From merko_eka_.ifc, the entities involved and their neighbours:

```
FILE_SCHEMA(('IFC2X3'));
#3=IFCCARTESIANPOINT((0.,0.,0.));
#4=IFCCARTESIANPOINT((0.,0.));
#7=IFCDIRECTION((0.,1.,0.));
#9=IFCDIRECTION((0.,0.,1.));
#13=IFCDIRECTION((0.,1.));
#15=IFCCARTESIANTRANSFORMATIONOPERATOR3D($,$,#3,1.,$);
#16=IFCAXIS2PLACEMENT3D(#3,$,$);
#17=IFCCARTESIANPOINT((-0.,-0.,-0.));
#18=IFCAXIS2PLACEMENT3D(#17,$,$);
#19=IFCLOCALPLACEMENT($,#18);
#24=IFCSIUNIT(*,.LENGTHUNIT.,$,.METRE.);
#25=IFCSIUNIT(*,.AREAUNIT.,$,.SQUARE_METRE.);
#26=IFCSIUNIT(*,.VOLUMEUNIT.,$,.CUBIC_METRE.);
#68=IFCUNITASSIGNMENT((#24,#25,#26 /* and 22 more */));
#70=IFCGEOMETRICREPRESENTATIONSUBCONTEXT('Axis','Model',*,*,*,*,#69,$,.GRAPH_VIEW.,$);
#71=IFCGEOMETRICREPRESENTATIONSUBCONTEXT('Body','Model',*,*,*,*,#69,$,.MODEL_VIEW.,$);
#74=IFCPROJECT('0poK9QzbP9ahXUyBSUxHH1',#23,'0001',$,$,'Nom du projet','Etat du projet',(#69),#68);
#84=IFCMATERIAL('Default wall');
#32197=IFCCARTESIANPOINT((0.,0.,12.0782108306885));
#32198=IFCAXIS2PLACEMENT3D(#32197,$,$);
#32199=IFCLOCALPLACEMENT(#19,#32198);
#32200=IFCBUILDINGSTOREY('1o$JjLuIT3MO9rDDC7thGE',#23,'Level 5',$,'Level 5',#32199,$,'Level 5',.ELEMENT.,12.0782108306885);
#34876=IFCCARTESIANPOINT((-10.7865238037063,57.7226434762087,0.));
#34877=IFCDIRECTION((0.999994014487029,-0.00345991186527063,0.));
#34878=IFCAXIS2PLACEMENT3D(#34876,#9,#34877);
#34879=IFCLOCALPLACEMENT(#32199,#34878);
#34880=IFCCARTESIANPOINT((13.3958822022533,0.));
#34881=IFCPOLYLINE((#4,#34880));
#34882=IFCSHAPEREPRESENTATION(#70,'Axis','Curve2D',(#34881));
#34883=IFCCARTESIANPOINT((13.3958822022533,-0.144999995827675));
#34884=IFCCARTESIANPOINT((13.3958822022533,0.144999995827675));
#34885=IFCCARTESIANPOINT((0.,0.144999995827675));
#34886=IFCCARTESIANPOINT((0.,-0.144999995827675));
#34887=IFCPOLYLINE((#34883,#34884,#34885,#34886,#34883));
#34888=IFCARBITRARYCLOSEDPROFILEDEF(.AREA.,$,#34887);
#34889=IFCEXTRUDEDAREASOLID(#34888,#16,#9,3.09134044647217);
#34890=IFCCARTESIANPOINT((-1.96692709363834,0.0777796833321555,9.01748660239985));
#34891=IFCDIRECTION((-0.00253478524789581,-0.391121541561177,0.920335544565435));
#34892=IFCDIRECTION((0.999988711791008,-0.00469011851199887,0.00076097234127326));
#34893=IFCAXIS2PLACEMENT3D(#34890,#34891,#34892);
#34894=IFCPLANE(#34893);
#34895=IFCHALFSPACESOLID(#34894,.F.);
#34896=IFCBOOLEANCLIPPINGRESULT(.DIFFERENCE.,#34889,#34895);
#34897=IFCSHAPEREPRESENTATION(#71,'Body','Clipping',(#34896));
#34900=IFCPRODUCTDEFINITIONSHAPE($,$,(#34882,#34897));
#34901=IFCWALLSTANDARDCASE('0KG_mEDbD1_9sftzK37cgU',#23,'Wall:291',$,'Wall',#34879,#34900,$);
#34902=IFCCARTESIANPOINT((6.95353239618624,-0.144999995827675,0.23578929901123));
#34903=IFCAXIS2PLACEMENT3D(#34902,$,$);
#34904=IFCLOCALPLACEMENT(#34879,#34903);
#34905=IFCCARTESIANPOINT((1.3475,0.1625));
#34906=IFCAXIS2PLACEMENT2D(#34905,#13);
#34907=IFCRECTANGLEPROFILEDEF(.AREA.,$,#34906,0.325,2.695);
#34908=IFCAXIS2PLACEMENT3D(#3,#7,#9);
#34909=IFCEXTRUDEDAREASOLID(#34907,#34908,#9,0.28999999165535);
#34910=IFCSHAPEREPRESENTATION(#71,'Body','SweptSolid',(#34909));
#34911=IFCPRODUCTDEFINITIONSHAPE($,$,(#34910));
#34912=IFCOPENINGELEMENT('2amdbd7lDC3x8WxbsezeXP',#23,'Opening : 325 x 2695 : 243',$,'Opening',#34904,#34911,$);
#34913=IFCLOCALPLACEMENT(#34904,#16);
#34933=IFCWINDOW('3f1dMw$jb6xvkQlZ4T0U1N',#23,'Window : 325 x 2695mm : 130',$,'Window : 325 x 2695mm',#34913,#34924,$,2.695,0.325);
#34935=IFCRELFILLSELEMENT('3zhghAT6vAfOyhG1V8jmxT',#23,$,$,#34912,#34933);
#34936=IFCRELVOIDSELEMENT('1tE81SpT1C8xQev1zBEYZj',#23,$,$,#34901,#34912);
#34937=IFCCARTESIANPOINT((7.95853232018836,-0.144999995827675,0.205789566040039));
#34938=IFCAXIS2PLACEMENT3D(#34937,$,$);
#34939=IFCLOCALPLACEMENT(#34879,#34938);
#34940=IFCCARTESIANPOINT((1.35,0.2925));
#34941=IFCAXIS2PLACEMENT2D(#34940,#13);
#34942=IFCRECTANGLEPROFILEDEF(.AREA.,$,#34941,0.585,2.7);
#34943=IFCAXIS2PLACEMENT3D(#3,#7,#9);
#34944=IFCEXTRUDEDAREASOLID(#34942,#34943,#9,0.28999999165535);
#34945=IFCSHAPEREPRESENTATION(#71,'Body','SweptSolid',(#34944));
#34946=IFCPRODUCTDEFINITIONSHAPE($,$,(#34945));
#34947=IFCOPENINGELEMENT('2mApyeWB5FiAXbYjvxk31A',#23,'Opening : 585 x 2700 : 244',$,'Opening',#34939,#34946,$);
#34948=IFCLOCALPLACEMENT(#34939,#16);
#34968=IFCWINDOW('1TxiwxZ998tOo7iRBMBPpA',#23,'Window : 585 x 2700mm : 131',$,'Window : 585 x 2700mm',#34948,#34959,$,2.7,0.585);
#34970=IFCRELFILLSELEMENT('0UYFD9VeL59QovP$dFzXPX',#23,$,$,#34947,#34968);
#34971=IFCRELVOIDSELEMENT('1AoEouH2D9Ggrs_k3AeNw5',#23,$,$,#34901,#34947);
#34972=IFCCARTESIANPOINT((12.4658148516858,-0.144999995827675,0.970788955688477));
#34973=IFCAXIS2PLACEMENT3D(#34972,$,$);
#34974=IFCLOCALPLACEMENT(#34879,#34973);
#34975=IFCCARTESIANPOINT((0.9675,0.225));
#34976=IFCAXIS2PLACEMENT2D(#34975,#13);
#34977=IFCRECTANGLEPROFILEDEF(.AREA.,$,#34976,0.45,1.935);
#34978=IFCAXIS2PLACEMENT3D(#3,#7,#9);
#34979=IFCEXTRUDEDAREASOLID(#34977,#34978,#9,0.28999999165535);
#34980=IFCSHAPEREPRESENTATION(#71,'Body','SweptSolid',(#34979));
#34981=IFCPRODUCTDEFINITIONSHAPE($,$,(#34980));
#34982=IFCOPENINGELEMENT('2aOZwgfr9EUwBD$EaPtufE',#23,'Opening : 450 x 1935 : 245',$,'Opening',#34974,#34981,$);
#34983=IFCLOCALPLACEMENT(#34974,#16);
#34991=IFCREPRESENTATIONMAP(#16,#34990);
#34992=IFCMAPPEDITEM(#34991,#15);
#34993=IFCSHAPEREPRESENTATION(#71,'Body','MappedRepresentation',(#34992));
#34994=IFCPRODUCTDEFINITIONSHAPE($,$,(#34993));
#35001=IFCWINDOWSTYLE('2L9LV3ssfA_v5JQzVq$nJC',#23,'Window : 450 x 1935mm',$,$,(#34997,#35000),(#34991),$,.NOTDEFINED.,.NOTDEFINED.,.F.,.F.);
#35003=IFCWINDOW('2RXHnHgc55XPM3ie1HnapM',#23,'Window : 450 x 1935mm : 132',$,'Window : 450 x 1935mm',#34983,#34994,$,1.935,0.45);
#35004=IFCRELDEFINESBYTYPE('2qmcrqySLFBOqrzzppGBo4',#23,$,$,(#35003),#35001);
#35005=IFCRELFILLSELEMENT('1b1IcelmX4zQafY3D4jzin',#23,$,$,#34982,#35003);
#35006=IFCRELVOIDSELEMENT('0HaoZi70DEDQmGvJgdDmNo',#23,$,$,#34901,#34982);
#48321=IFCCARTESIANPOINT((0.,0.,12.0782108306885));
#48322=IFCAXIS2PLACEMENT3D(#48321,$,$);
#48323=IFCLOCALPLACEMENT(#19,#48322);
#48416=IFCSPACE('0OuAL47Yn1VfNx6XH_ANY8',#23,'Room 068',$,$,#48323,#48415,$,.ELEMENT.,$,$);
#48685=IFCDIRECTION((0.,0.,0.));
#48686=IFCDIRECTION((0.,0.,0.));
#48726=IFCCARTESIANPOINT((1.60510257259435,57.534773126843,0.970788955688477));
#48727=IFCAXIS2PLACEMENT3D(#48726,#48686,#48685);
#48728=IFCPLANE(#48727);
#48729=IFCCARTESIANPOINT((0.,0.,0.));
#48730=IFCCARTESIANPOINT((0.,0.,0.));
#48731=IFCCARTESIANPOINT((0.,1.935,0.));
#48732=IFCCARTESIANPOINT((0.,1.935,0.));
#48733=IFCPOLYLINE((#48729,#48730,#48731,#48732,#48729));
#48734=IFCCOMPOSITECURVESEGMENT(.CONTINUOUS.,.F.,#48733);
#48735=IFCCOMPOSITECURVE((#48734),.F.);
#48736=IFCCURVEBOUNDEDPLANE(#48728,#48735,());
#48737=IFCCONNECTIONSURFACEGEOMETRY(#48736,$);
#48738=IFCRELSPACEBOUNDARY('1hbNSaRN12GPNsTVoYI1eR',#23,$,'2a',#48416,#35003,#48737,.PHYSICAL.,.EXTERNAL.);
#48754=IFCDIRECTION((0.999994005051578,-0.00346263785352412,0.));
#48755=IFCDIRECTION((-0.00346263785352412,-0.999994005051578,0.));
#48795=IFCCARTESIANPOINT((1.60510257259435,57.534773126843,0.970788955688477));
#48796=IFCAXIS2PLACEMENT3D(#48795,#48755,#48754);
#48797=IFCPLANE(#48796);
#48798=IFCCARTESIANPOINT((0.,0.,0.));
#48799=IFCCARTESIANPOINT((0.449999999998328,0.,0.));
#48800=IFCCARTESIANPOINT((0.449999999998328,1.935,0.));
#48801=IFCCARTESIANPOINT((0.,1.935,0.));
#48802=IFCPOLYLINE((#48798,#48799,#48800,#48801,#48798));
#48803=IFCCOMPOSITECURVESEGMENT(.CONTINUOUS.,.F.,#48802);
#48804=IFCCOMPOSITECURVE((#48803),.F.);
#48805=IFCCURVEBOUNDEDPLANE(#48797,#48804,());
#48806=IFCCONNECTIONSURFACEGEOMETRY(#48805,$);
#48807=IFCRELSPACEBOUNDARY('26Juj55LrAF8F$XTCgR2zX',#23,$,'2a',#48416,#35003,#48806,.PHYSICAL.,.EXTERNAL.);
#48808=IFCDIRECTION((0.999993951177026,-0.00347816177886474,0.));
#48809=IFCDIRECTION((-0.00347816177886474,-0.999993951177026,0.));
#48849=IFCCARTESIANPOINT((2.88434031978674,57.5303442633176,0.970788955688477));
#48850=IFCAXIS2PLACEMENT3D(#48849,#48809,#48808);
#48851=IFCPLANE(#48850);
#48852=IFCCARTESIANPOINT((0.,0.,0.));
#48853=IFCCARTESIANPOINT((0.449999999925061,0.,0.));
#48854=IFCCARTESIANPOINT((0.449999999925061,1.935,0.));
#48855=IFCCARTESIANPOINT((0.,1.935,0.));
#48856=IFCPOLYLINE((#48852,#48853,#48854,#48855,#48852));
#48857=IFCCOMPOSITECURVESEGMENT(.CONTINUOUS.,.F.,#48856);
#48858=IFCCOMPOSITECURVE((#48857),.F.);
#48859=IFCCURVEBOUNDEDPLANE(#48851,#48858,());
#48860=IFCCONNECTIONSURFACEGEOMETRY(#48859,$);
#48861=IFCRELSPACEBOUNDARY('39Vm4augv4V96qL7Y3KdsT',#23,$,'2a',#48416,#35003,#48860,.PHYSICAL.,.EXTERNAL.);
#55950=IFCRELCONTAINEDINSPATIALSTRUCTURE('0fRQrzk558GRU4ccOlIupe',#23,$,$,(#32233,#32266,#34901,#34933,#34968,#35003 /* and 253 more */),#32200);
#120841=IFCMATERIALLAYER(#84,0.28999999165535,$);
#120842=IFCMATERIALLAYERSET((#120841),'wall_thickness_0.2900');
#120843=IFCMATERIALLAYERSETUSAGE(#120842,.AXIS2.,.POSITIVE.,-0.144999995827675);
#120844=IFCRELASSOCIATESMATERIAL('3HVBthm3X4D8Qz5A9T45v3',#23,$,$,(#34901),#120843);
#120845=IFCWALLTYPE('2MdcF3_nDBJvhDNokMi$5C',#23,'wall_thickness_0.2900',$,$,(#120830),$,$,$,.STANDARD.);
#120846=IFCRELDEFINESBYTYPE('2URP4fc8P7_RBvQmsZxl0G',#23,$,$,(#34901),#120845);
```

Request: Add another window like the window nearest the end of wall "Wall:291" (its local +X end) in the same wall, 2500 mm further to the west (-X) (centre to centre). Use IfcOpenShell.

```python
import numpy as np
import ifcopenshell
import ifcopenshell.api.feature
import ifcopenshell.api.geometry
import ifcopenshell.api.root
import ifcopenshell.geom
import ifcopenshell.util.element
import ifcopenshell.util.placement
import ifcopenshell.util.shape
import ifcopenshell.util.unit

model = ifcopenshell.open("merko_eka_.ifc")
unit_scale = ifcopenshell.util.unit.calculate_unit_scale(model)
settings = ifcopenshell.geom.settings()


def volume(element):
    """Net volume in cubic metres, openings subtracted."""
    shape = ifcopenshell.geom.create_shape(settings, element)
    return ifcopenshell.util.shape.get_volume(shape.geometry)


window = model.by_id(35003)
opening = window.FillsVoids[0].RelatingOpeningElement
wall = opening.VoidsElements[0].RelatingBuildingElement
before = volume(wall)
shift = ifcopenshell.util.placement.get_local_placement(wall.ObjectPlacement)[:3, 0] * -2.5 / unit_scale

# copy_class copies the void relationship, type, container and properties, but no geometry.
new_opening = ifcopenshell.api.root.copy_class(model, product=opening)
new_opening.Representation = ifcopenshell.util.element.copy_deep(
    model, opening.Representation, exclude=["IfcGeometricRepresentationContext", "IfcRepresentationMap"]
)
new_opening.Name = "Opening : 450 x 1935"
new_window = ifcopenshell.api.root.copy_class(model, product=window)
new_window.Representation = ifcopenshell.util.element.copy_deep(
    model, window.Representation, exclude=["IfcGeometricRepresentationContext", "IfcRepresentationMap"]
)
new_window.Name = "Window : 450 x 1935mm"
fills = ifcopenshell.api.feature.add_filling(model, opening=new_opening, element=new_window)
fills.OwnerHistory = new_window.OwnerHistory  # required in IFC2X3

for old, new in ((opening, new_opening), (window, new_window)):
    matrix = ifcopenshell.util.placement.get_local_placement(old.ObjectPlacement)
    matrix[:3, 3] += shift
    ifcopenshell.api.geometry.edit_object_placement(model, product=new, matrix=matrix, is_si=False)

# The copied space boundaries still share their surfaces with the original.
for rel in new_window.ProvidesBoundaries:
    if rel.ConnectionGeometry:
        rel.ConnectionGeometry = ifcopenshell.util.element.copy_deep(model, rel.ConnectionGeometry)

# Space boundary surfaces are stored in each space's coordinates; move them too.
for rel in new_window.ProvidesBoundaries:
    if not rel.ConnectionGeometry:
        continue
    surface = rel.ConnectionGeometry.SurfaceOnRelatingElement.BasisSurface
    space_matrix = ifcopenshell.util.placement.get_local_placement(rel.RelatingSpace.ObjectPlacement)
    point = np.array(surface.Position.Location.Coordinates) + space_matrix[:3, :3].T @ shift
    surface.Position = model.createIfcAxis2Placement3D(
        model.createIfcCartesianPoint(point.tolist()), surface.Position.Axis, surface.Position.RefDirection
    )

after = volume(wall)

print(f"wall volume {before:.3f} -> {after:.3f} m3")

model.write("merko_eka__v2.ifc")
```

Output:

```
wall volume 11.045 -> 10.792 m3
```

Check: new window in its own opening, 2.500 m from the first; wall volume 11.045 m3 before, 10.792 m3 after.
